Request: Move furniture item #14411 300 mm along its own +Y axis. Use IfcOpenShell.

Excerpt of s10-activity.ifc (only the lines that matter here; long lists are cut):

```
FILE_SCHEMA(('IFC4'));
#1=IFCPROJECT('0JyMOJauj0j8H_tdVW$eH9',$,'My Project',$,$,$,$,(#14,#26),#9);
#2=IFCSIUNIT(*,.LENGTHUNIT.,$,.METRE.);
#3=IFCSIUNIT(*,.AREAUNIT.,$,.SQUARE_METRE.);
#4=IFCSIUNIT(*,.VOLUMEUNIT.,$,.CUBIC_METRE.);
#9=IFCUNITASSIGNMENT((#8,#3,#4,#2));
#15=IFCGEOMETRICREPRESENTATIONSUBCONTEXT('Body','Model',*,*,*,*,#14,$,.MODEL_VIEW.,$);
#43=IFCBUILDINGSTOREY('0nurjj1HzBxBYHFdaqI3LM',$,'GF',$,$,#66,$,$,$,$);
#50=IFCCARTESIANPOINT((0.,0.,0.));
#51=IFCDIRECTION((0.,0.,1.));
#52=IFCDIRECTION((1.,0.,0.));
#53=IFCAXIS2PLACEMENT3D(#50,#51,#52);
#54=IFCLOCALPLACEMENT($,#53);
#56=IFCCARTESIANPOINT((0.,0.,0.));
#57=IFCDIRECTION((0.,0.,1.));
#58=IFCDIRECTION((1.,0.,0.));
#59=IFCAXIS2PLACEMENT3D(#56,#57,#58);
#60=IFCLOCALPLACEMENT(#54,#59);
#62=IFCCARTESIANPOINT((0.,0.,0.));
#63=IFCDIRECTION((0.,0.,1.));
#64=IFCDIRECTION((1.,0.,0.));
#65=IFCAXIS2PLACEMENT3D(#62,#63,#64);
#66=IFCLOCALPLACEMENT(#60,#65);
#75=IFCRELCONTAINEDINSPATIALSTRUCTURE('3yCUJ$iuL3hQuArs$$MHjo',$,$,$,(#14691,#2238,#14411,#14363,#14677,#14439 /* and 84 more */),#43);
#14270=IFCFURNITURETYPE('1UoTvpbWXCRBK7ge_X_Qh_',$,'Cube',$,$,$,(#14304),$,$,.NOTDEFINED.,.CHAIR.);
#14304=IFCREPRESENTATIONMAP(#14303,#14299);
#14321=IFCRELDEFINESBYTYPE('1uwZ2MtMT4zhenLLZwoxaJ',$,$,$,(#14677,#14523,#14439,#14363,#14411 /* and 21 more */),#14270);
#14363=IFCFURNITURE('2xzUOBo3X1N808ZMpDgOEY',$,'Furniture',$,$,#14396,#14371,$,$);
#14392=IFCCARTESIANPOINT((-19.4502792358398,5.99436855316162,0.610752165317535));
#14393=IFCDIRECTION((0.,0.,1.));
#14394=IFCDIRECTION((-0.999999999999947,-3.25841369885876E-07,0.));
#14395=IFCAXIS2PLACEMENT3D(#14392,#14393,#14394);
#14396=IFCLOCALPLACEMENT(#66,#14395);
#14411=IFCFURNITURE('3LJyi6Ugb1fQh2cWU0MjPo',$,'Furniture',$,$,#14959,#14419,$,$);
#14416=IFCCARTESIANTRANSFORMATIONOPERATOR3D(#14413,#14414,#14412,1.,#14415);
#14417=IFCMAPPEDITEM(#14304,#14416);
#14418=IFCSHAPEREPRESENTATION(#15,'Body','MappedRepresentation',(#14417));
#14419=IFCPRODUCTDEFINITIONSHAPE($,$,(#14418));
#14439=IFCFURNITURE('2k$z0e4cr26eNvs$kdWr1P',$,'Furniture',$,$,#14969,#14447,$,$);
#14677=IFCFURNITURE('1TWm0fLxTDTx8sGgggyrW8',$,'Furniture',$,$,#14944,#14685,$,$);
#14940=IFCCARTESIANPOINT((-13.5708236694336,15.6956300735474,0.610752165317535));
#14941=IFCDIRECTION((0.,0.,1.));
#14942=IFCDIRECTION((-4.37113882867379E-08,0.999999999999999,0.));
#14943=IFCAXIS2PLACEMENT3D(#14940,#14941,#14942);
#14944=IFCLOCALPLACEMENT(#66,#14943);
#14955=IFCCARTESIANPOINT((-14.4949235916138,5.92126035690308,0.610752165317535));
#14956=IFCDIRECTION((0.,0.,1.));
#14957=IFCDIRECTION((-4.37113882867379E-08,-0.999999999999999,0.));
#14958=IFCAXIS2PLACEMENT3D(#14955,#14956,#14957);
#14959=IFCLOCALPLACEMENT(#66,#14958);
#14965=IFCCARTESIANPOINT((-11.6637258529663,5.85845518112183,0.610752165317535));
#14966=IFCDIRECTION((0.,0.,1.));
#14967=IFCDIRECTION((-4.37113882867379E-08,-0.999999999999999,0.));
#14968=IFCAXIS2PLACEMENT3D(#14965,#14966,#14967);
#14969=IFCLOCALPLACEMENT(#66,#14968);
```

```python
import ifcopenshell
import ifcopenshell.api.geometry
import ifcopenshell.util.placement

model = ifcopenshell.open("s10-activity.ifc")

item = model.by_guid("3LJyi6Ugb1fQh2cWU0MjPo")
matrix = ifcopenshell.util.placement.get_local_placement(item.ObjectPlacement)
matrix[:3, 3] += matrix[:3, 1] * 0.3
ifcopenshell.api.geometry.edit_object_placement(model, product=item, matrix=matrix, is_si=False)

print(ifcopenshell.util.placement.get_local_placement(item.ObjectPlacement).round(3) + 0.0)

model.write("s10-activity_rev.ifc")
```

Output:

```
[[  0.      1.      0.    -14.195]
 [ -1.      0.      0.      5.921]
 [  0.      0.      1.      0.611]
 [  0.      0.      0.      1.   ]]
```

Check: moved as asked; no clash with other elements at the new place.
